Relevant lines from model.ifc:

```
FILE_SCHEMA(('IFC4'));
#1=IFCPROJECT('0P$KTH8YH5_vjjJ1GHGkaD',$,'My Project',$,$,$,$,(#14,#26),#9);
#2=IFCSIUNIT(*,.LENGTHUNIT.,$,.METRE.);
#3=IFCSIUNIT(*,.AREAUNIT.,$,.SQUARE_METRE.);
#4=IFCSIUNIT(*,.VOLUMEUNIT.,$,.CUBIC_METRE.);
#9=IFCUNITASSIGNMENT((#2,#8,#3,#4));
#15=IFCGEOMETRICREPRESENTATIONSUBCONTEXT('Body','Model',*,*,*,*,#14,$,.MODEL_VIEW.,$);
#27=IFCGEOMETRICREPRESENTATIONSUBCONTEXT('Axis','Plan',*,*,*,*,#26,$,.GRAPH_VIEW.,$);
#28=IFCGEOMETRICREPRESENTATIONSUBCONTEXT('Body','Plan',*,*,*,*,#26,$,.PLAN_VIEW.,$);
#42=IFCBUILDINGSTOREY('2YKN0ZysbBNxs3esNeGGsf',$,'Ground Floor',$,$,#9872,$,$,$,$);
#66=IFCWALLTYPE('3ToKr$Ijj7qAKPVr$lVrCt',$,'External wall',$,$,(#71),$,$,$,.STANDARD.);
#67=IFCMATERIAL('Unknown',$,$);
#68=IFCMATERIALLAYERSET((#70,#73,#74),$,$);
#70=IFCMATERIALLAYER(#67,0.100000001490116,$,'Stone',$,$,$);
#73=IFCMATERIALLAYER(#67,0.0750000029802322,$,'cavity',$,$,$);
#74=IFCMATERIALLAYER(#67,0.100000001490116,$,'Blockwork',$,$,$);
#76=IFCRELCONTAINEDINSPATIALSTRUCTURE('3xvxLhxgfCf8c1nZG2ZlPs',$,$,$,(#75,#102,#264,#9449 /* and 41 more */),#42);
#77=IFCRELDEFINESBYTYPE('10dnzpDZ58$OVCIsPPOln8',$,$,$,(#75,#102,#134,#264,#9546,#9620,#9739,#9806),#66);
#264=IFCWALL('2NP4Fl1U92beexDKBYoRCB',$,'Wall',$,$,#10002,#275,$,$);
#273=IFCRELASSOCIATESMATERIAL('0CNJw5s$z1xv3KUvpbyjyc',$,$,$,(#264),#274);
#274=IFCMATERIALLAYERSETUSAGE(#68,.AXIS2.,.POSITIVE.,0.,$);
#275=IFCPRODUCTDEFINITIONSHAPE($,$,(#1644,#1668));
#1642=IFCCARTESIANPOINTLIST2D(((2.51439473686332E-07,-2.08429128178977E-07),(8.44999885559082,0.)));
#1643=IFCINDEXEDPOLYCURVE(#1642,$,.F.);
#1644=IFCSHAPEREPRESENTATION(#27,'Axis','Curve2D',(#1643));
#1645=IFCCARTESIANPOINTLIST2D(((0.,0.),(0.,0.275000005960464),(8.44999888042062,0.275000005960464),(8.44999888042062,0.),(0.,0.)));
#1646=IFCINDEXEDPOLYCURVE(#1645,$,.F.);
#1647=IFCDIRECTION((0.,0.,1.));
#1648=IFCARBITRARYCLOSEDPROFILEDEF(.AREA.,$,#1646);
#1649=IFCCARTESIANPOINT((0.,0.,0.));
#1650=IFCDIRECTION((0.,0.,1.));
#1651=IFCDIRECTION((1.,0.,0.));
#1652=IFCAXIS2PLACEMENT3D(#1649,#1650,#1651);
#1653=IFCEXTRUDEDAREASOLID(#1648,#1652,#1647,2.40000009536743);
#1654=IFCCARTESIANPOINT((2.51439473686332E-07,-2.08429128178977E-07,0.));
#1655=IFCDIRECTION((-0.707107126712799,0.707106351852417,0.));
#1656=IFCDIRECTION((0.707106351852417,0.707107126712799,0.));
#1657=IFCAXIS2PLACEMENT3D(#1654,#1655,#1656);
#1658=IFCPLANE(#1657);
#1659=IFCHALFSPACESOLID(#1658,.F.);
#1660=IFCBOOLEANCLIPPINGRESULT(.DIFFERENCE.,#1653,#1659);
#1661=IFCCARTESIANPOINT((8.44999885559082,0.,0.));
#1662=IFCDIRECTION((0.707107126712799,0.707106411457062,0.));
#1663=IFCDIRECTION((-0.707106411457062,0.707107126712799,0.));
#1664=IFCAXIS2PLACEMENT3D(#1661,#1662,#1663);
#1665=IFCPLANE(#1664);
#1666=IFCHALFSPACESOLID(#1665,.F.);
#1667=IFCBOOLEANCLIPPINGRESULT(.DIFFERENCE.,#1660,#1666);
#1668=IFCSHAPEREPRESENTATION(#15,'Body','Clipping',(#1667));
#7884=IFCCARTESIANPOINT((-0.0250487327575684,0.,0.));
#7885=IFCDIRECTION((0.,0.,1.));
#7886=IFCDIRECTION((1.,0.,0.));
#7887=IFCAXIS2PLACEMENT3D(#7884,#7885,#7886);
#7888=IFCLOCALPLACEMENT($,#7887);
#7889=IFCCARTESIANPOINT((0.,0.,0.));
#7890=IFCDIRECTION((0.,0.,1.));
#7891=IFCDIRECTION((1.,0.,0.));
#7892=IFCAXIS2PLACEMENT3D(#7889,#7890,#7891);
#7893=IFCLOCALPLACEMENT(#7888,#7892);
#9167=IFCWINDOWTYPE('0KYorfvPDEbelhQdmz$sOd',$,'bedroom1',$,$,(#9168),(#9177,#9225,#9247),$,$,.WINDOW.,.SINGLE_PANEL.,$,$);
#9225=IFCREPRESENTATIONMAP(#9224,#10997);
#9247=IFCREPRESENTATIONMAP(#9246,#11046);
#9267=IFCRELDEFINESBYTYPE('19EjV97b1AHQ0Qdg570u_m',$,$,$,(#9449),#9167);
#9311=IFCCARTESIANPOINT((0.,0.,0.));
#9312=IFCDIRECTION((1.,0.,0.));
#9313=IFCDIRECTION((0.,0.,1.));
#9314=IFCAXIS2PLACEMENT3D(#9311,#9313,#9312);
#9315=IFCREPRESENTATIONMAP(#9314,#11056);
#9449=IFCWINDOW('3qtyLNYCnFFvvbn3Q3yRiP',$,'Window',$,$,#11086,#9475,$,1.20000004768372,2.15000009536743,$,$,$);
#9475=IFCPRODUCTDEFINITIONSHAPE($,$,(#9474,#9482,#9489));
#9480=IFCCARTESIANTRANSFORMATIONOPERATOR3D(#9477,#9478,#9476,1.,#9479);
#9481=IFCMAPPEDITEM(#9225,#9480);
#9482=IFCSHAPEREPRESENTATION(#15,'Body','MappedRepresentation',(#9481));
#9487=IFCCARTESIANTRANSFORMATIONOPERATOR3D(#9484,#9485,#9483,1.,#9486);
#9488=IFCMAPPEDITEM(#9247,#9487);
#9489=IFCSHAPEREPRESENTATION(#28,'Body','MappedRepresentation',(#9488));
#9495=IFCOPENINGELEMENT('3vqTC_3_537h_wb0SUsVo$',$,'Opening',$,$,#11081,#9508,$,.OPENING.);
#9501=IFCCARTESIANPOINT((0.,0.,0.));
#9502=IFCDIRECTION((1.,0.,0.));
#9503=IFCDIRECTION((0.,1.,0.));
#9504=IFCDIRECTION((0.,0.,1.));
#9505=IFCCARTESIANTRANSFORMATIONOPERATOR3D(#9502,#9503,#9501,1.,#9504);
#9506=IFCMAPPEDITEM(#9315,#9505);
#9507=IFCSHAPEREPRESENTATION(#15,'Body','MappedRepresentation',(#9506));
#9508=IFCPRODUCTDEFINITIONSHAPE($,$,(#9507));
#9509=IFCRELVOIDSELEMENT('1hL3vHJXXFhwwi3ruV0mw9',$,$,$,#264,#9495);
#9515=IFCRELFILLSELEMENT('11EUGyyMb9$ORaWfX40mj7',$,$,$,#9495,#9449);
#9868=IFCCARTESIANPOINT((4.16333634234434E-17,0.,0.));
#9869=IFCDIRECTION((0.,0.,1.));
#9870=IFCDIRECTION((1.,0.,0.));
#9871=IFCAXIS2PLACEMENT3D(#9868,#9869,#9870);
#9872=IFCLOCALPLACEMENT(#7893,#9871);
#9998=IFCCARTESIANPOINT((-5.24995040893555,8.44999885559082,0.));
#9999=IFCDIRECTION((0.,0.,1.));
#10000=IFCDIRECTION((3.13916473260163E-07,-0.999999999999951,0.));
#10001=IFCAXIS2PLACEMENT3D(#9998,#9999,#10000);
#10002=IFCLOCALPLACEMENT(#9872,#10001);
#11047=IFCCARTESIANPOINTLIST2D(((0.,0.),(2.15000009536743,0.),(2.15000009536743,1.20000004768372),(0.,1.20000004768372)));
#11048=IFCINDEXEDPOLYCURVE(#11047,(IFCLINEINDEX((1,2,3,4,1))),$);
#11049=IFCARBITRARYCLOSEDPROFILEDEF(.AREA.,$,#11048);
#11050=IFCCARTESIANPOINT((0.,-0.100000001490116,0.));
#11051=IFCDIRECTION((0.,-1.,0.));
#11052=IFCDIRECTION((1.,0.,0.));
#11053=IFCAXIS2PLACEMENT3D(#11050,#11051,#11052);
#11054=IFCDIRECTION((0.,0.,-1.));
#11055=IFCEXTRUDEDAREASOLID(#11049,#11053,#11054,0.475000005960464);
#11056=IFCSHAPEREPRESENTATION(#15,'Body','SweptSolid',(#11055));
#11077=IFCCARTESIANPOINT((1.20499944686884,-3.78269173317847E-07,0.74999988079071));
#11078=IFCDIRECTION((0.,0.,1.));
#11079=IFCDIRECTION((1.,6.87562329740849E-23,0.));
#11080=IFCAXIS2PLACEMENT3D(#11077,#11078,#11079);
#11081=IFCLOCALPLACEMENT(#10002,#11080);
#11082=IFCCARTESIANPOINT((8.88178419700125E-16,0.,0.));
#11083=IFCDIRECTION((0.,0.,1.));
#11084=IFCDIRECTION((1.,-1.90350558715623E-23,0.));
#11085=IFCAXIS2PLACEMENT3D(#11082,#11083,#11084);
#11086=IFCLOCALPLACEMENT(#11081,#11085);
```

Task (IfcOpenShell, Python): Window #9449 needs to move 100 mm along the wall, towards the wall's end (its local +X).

```python
import ifcopenshell
import ifcopenshell.api.geometry
import ifcopenshell.util.placement

model = ifcopenshell.open("model.ifc")

window = model.by_guid("3qtyLNYCnFFvvbn3Q3yRiP")
opening = window.FillsVoids[0].RelatingOpeningElement
wall = opening.VoidsElements[0].RelatingBuildingElement

wall_matrix = ifcopenshell.util.placement.get_local_placement(wall.ObjectPlacement)
shift = wall_matrix[:3, 0] * 0.1
before = ifcopenshell.util.placement.get_local_placement(window.ObjectPlacement)[:3, 3].copy()

# The window is placed relative to its opening, so it follows when the opening moves.
matrix = ifcopenshell.util.placement.get_local_placement(opening.ObjectPlacement)
matrix[:3, 3] += shift
ifcopenshell.api.geometry.edit_object_placement(
    model, product=opening, matrix=matrix, is_si=False, should_transform_children=True
)

after = ifcopenshell.util.placement.get_local_placement(window.ObjectPlacement)[:3, 3]
print("window moved by", (after - before).round(3) + 0.0)

model.write("model_rev.ifc")
```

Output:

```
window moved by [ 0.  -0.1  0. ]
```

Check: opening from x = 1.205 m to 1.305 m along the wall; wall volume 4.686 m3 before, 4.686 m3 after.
